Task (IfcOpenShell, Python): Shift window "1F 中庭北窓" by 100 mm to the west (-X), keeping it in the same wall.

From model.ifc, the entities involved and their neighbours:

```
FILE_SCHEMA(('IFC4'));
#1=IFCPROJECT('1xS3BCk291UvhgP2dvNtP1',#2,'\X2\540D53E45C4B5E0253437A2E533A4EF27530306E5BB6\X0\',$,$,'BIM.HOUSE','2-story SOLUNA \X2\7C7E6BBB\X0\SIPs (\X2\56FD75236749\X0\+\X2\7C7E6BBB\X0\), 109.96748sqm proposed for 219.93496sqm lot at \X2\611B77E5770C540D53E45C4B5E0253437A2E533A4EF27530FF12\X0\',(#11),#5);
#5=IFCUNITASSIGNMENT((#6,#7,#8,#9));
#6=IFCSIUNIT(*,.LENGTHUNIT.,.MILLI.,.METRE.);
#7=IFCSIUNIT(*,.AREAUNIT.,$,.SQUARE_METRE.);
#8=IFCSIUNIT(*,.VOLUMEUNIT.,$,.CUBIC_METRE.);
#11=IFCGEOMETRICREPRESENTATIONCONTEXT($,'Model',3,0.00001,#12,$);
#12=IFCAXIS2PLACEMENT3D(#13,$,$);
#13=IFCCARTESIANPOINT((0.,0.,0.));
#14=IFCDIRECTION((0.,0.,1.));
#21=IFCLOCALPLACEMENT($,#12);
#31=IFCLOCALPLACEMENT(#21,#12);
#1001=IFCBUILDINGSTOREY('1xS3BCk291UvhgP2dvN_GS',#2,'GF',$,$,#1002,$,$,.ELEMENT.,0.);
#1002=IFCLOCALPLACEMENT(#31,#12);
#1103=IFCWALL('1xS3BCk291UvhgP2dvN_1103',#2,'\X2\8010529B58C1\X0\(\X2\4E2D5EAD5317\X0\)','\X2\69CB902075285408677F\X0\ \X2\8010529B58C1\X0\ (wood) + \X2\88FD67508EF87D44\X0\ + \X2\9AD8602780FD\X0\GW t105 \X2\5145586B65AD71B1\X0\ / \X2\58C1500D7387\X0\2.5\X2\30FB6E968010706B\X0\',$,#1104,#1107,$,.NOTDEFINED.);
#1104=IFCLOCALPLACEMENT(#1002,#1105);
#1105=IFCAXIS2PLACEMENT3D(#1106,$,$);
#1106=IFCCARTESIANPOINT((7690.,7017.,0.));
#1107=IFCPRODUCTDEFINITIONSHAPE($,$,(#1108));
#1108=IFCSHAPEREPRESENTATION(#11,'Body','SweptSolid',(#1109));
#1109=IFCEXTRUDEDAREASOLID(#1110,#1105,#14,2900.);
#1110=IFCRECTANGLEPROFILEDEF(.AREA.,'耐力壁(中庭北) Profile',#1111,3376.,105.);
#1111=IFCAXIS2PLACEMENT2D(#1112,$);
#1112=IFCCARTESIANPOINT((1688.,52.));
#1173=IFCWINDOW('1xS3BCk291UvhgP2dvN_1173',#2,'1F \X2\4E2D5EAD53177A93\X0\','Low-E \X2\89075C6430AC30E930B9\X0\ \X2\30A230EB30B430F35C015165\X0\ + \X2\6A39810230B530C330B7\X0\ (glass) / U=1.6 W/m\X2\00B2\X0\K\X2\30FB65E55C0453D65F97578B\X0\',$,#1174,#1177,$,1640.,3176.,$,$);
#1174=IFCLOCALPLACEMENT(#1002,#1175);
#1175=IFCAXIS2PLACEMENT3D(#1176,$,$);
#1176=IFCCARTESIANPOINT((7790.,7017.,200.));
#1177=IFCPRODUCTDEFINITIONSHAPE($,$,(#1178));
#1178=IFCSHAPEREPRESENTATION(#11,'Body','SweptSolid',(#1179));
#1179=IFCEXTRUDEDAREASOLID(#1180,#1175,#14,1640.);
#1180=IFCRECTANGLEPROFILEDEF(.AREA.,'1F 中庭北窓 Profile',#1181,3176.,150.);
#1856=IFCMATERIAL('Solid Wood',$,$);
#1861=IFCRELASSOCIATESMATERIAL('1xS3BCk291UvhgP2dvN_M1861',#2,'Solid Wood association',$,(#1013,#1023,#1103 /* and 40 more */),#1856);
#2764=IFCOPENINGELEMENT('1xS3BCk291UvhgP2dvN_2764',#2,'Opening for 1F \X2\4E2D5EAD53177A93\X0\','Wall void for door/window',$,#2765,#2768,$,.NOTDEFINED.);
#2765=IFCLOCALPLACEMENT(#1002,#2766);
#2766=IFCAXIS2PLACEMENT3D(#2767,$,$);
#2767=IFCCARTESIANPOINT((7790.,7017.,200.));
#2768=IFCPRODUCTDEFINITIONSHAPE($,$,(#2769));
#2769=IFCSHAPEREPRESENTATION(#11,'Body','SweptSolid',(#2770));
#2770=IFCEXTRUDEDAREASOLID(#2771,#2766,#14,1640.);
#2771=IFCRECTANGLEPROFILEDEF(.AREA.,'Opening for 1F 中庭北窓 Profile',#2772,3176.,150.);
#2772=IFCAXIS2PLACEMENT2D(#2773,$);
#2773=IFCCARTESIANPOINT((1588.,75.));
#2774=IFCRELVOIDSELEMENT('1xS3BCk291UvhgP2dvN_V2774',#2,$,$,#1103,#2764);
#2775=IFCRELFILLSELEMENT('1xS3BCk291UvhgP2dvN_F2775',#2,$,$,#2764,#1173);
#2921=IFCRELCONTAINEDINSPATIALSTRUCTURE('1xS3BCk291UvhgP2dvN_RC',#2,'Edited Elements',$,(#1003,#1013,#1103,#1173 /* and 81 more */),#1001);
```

```python
import ifcopenshell
import ifcopenshell.api.geometry
import ifcopenshell.util.placement
import ifcopenshell.util.unit

model = ifcopenshell.open("model.ifc")
unit_scale = ifcopenshell.util.unit.calculate_unit_scale(model)

window = model.by_id(1173)
opening = window.FillsVoids[0].RelatingOpeningElement
wall = opening.VoidsElements[0].RelatingBuildingElement

wall_matrix = ifcopenshell.util.placement.get_local_placement(wall.ObjectPlacement)
shift = wall_matrix[:3, 0] * -0.1 / unit_scale
before = ifcopenshell.util.placement.get_local_placement(window.ObjectPlacement)[:3, 3].copy()

# The window is not placed relative to its opening, so move both.
for product in (opening, window):
    matrix = ifcopenshell.util.placement.get_local_placement(product.ObjectPlacement)
    matrix[:3, 3] += shift
    ifcopenshell.api.geometry.edit_object_placement(model, product=product, matrix=matrix, is_si=False)

after = ifcopenshell.util.placement.get_local_placement(window.ObjectPlacement)[:3, 3]
print("window moved by", (after - before).round(3) + 0.0)

model.write("model-out.ifc")
```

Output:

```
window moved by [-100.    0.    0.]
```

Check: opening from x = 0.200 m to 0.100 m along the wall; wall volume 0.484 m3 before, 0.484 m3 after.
